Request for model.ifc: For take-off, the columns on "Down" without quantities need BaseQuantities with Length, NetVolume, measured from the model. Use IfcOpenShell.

First a look at what the model holds.

```python
import ifcopenshell
import ifcopenshell.util.element
import ifcopenshell.util.unit

model = ifcopenshell.open("model.ifc")
print(model.schema)
for unit_type in ("LENGTHUNIT", "AREAUNIT", "VOLUMEUNIT"):
    print(unit_type, ifcopenshell.util.unit.calculate_unit_scale(model, unit_type))
storey = next(s for s in model.by_type("IfcBuildingStorey") if s.Name == "Down")
columns = [e for e in ifcopenshell.util.element.get_decomposition(storey) if e.is_a("IfcColumn")]
for e in sorted(columns, key=lambda e: e.id()):
    print(e.id(), e.is_a(), e.Name, list(ifcopenshell.util.element.get_psets(e, qtos_only=True)), sep=" | ")
```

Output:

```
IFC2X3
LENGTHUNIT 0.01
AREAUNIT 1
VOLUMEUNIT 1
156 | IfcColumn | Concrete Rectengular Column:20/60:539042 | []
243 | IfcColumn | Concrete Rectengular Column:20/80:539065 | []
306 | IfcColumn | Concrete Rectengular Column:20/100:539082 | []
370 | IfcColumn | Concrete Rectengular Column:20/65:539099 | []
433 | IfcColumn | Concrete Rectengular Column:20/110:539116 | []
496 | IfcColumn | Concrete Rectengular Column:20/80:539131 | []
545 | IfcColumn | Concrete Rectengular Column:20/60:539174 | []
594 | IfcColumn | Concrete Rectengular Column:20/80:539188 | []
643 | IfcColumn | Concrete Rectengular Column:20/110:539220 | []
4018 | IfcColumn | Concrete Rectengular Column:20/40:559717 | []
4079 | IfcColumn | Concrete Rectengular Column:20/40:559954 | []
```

```python
import ifcopenshell
import ifcopenshell.api.pset
import ifcopenshell.geom
import ifcopenshell.util.element
import ifcopenshell.util.shape
import ifcopenshell.util.unit

model = ifcopenshell.open("model.ifc")
unit_scale = ifcopenshell.util.unit.calculate_unit_scale(model)
volume_scale = ifcopenshell.util.unit.calculate_unit_scale(model, "VOLUMEUNIT")
settings = ifcopenshell.geom.settings()

storey = next(s for s in model.by_type("IfcBuildingStorey") if s.Name == "Down")
columns = [e for e in ifcopenshell.util.element.get_decomposition(storey) if e.is_a("IfcColumn")]

for e in sorted(columns, key=lambda e: e.id()):
    if ifcopenshell.util.element.get_psets(e, qtos_only=True, should_inherit=False):
        continue
    # Geometry comes back in metres, in the element's own axes.
    shape = ifcopenshell.geom.create_shape(settings, e)
    values = {
        "Length": ifcopenshell.util.shape.get_z(shape.geometry) / unit_scale,
        "NetVolume": ifcopenshell.util.shape.get_volume(shape.geometry) / volume_scale,
    }
    qto = ifcopenshell.api.pset.add_qto(model, product=e, name="BaseQuantities")
    ifcopenshell.api.pset.edit_qto(model, qto=qto, properties=values)
    print(e.id(), {k: round(v, 3) for k, v in values.items()})

model.write("model_updated.ifc")
```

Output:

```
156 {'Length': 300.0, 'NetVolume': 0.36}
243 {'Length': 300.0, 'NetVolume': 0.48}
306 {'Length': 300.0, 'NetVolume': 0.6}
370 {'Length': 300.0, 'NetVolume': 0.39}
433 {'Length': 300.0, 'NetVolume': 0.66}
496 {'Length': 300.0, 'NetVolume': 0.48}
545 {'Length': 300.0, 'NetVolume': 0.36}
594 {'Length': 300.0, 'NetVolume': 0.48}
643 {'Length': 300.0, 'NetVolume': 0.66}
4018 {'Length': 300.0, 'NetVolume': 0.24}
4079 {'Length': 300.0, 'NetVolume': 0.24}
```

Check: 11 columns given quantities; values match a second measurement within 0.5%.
